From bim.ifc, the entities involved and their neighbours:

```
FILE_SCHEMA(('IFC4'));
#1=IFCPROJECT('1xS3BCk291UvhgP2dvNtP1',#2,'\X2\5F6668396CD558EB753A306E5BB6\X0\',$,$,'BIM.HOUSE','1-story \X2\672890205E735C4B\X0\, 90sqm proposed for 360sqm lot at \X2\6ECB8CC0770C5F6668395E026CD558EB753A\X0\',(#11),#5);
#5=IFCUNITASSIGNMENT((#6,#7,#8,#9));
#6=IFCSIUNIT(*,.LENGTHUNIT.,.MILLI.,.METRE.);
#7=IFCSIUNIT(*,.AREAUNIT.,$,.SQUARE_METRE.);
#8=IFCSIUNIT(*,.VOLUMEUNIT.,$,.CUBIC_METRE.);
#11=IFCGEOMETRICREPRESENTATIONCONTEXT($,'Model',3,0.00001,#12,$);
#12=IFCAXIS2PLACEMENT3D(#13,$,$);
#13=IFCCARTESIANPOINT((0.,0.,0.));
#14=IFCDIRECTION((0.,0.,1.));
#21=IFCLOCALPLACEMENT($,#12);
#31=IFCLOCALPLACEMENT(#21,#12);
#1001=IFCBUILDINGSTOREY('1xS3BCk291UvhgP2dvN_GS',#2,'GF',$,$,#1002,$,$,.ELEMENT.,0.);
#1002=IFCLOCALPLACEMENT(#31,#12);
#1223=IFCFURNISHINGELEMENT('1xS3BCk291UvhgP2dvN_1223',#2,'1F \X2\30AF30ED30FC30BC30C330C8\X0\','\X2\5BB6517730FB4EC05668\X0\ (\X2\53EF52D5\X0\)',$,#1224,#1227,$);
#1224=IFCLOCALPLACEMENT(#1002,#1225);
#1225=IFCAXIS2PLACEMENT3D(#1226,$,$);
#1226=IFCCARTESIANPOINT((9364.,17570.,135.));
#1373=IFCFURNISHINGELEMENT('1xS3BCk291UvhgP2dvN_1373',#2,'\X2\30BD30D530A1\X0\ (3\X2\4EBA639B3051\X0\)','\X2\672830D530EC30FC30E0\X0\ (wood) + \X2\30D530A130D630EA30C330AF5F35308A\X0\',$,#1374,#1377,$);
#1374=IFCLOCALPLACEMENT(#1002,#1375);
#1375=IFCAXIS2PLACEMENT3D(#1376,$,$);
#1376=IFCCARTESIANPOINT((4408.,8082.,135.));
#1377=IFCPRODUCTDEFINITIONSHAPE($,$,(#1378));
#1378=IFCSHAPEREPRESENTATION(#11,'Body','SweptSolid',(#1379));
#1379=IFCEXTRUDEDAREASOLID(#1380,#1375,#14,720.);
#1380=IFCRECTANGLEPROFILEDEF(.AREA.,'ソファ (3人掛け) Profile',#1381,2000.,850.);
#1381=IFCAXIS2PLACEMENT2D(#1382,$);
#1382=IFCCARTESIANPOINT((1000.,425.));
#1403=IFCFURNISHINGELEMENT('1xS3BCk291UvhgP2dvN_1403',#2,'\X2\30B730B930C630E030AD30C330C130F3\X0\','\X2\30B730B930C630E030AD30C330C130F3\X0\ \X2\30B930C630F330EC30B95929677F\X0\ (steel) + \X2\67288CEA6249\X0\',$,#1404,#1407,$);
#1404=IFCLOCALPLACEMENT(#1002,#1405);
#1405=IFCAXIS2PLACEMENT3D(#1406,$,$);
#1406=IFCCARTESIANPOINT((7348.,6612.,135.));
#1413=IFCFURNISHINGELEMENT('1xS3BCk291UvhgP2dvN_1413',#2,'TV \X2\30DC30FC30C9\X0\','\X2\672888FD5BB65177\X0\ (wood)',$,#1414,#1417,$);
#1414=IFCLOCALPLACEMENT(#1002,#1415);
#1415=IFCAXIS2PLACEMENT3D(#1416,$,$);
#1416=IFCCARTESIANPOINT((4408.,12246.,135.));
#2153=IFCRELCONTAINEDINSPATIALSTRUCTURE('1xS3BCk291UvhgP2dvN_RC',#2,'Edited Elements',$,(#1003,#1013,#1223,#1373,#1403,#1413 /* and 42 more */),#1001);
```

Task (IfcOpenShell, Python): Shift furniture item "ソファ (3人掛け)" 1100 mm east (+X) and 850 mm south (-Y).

```python
import ifcopenshell
import ifcopenshell.api.geometry
import ifcopenshell.util.placement
import ifcopenshell.util.unit

model = ifcopenshell.open("bim.ifc")
unit_scale = ifcopenshell.util.unit.calculate_unit_scale(model)

item = model.by_guid("1xS3BCk291UvhgP2dvN_1373")
matrix = ifcopenshell.util.placement.get_local_placement(item.ObjectPlacement)
matrix[0, 3] += 1.1 / unit_scale
matrix[1, 3] -= 0.85 / unit_scale
ifcopenshell.api.geometry.edit_object_placement(model, product=item, matrix=matrix, is_si=False)

print(ifcopenshell.util.placement.get_local_placement(item.ObjectPlacement).round(3) + 0.0)

model.write("bim_updated.ifc")
```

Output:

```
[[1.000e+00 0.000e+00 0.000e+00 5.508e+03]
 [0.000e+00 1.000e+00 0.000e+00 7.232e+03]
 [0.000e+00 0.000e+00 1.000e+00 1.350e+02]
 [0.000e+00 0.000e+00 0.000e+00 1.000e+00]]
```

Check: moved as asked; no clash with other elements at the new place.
